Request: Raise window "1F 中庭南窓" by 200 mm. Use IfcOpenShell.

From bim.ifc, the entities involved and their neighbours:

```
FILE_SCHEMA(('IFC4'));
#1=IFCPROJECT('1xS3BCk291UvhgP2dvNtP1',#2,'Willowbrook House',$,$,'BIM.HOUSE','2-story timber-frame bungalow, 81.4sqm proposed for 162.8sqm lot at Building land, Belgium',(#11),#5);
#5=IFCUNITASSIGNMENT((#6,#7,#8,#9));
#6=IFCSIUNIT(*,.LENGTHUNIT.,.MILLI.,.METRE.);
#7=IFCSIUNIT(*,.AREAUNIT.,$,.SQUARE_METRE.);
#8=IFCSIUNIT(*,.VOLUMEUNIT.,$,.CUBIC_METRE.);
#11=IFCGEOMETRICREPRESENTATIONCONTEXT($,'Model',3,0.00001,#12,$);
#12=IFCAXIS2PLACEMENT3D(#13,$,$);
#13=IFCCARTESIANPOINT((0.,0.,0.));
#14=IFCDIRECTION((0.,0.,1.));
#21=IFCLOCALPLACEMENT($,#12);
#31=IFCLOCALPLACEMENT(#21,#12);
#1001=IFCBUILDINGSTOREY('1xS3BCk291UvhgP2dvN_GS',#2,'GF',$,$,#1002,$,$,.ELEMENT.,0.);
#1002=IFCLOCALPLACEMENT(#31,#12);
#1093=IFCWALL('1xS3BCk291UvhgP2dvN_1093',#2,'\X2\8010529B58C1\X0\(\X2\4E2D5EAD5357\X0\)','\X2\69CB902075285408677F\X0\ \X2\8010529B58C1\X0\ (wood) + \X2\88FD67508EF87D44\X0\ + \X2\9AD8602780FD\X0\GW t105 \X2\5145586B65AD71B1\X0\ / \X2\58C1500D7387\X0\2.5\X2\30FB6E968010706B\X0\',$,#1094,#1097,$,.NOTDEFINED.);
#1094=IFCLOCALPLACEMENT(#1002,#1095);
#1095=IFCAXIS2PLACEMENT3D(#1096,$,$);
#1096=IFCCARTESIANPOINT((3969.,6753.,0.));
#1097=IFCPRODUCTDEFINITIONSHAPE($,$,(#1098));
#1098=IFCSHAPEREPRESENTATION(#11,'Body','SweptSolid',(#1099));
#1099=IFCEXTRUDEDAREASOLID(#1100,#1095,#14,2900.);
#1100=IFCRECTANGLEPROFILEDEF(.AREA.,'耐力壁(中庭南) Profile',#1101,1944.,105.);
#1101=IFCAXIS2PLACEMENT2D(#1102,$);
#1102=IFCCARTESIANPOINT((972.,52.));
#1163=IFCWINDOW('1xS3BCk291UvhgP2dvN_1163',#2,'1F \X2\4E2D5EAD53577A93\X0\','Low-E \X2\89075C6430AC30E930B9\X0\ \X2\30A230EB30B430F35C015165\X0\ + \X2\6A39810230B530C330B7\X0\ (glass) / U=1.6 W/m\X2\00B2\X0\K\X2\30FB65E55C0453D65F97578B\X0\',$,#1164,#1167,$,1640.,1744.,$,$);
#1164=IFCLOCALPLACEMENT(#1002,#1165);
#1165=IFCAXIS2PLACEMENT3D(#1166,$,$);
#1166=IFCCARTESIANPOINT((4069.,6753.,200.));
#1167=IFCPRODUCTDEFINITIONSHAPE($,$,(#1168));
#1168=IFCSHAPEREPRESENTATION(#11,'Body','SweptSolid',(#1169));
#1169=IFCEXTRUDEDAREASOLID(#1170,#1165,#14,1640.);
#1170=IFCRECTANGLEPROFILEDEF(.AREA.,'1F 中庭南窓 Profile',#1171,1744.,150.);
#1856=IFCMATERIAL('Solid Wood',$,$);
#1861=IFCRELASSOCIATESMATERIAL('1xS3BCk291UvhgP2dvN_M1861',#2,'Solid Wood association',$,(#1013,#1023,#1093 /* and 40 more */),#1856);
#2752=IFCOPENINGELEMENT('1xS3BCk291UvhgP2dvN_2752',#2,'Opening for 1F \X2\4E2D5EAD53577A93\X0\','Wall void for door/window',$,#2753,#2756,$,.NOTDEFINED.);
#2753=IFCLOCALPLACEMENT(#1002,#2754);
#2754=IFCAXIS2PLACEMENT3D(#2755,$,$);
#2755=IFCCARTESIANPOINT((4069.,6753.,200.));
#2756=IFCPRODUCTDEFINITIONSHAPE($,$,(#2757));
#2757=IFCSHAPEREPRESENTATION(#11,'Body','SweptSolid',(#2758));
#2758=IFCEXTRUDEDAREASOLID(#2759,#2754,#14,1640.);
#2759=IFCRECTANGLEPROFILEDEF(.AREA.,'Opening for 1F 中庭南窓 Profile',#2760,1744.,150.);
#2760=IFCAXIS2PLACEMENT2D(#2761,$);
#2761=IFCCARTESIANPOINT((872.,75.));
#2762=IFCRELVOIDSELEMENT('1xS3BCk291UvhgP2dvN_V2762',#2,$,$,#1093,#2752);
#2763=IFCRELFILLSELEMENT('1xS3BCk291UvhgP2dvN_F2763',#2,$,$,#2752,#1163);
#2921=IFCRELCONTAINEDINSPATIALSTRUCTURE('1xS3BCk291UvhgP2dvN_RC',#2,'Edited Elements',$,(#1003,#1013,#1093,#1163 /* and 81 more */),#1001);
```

```python
import numpy as np
import ifcopenshell
import ifcopenshell.api.geometry
import ifcopenshell.util.placement
import ifcopenshell.util.unit

model = ifcopenshell.open("bim.ifc")
unit_scale = ifcopenshell.util.unit.calculate_unit_scale(model)

window = model.by_id(1163)
opening = window.FillsVoids[0].RelatingOpeningElement
dz = 0.2 / unit_scale

shift = np.array([0.0, 0.0, dz])
# The window is not placed relative to its opening, so move both.
for product in (opening, window):
    matrix = ifcopenshell.util.placement.get_local_placement(product.ObjectPlacement)
    matrix[:3, 3] += shift
    ifcopenshell.api.geometry.edit_object_placement(model, product=product, matrix=matrix, is_si=False)

print(f"moved by {dz * unit_scale:+.3f} m")

model.write("bim_v2.ifc")
```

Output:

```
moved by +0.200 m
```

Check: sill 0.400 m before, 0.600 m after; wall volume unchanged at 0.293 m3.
